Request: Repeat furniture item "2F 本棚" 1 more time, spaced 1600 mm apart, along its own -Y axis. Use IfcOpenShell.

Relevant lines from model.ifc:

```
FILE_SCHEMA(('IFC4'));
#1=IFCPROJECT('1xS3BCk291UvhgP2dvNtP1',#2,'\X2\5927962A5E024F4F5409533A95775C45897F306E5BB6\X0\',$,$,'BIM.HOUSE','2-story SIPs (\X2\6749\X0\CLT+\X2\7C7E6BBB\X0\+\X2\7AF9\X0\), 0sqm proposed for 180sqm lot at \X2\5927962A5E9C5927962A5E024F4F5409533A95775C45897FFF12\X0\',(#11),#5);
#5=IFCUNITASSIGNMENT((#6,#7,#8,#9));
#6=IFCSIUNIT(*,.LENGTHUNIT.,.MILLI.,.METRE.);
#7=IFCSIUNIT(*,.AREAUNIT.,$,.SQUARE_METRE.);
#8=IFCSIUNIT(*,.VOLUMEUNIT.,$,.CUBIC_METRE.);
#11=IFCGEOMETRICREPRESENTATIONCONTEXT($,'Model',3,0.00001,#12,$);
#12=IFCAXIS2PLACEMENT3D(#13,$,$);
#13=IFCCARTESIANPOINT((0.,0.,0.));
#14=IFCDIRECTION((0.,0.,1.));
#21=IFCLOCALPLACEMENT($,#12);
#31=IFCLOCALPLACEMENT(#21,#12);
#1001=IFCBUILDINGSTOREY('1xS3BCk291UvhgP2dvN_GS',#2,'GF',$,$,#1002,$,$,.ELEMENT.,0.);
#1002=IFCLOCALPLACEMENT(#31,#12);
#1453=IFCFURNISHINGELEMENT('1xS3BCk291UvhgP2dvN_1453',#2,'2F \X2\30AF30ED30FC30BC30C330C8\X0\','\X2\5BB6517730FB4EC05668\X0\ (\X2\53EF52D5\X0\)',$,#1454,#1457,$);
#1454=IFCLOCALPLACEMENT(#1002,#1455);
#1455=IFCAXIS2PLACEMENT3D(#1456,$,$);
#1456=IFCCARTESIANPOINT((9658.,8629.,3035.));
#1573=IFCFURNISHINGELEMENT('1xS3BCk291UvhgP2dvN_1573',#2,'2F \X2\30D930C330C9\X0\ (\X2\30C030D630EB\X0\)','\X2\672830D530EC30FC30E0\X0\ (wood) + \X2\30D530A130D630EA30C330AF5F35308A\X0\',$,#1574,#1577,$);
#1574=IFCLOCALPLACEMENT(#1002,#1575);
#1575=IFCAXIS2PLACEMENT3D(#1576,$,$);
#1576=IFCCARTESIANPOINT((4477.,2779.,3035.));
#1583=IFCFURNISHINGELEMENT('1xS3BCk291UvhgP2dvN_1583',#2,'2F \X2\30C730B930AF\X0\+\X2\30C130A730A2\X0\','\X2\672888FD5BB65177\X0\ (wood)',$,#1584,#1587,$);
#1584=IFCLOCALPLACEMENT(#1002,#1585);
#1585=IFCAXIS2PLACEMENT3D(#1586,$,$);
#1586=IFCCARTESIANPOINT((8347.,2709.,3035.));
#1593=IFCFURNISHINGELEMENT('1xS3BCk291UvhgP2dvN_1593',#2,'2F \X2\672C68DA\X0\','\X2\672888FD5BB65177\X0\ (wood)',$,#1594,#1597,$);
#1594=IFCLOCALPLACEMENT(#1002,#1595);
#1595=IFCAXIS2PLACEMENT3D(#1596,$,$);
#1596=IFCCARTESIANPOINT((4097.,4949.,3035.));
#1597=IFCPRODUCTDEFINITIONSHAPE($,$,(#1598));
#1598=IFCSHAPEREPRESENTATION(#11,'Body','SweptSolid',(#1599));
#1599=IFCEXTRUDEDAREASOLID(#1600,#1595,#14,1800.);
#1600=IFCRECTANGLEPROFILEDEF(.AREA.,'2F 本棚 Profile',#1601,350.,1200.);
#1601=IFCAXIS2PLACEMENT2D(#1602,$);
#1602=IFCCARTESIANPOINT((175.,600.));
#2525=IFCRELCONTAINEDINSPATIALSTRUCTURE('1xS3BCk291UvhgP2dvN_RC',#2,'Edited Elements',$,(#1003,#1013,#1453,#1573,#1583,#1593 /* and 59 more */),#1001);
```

```python
import ifcopenshell
import ifcopenshell.api.geometry
import ifcopenshell.api.root
import ifcopenshell.util.element
import ifcopenshell.util.placement
import ifcopenshell.util.unit

model = ifcopenshell.open("model.ifc")
unit_scale = ifcopenshell.util.unit.calculate_unit_scale(model)


def reuse_history(source, copy):
    """copy_class also copies each property set's owner history, people and application; keep the originals."""
    for rel in copy.IsDefinedBy:
        if rel.is_a("IfcRelDefinesByProperties") and (history := rel.RelatingPropertyDefinition.OwnerHistory):
            rel.RelatingPropertyDefinition.OwnerHistory = source.OwnerHistory
            ifcopenshell.util.element.remove_deep2(model, history)


source = model.by_id(1593)
base = ifcopenshell.util.placement.get_local_placement(source.ObjectPlacement)
step = -base[:3, 1] * 1.6 / unit_scale

for i in range(1, 2):
    copy = ifcopenshell.api.root.copy_class(model, product=source)
    copy.Representation = ifcopenshell.util.element.copy_deep(
        model, source.Representation, exclude=["IfcGeometricRepresentationContext", "IfcRepresentationMap"]
    )
    reuse_history(source, copy)
    matrix = base.copy()
    matrix[:3, 3] += i * step
    print("added at", matrix[:3, 3].round(3) + 0.0)
    ifcopenshell.api.geometry.edit_object_placement(model, product=copy, matrix=matrix, is_si=False)

model.write("model_rev.ifc")
```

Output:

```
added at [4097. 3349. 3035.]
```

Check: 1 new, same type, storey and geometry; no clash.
